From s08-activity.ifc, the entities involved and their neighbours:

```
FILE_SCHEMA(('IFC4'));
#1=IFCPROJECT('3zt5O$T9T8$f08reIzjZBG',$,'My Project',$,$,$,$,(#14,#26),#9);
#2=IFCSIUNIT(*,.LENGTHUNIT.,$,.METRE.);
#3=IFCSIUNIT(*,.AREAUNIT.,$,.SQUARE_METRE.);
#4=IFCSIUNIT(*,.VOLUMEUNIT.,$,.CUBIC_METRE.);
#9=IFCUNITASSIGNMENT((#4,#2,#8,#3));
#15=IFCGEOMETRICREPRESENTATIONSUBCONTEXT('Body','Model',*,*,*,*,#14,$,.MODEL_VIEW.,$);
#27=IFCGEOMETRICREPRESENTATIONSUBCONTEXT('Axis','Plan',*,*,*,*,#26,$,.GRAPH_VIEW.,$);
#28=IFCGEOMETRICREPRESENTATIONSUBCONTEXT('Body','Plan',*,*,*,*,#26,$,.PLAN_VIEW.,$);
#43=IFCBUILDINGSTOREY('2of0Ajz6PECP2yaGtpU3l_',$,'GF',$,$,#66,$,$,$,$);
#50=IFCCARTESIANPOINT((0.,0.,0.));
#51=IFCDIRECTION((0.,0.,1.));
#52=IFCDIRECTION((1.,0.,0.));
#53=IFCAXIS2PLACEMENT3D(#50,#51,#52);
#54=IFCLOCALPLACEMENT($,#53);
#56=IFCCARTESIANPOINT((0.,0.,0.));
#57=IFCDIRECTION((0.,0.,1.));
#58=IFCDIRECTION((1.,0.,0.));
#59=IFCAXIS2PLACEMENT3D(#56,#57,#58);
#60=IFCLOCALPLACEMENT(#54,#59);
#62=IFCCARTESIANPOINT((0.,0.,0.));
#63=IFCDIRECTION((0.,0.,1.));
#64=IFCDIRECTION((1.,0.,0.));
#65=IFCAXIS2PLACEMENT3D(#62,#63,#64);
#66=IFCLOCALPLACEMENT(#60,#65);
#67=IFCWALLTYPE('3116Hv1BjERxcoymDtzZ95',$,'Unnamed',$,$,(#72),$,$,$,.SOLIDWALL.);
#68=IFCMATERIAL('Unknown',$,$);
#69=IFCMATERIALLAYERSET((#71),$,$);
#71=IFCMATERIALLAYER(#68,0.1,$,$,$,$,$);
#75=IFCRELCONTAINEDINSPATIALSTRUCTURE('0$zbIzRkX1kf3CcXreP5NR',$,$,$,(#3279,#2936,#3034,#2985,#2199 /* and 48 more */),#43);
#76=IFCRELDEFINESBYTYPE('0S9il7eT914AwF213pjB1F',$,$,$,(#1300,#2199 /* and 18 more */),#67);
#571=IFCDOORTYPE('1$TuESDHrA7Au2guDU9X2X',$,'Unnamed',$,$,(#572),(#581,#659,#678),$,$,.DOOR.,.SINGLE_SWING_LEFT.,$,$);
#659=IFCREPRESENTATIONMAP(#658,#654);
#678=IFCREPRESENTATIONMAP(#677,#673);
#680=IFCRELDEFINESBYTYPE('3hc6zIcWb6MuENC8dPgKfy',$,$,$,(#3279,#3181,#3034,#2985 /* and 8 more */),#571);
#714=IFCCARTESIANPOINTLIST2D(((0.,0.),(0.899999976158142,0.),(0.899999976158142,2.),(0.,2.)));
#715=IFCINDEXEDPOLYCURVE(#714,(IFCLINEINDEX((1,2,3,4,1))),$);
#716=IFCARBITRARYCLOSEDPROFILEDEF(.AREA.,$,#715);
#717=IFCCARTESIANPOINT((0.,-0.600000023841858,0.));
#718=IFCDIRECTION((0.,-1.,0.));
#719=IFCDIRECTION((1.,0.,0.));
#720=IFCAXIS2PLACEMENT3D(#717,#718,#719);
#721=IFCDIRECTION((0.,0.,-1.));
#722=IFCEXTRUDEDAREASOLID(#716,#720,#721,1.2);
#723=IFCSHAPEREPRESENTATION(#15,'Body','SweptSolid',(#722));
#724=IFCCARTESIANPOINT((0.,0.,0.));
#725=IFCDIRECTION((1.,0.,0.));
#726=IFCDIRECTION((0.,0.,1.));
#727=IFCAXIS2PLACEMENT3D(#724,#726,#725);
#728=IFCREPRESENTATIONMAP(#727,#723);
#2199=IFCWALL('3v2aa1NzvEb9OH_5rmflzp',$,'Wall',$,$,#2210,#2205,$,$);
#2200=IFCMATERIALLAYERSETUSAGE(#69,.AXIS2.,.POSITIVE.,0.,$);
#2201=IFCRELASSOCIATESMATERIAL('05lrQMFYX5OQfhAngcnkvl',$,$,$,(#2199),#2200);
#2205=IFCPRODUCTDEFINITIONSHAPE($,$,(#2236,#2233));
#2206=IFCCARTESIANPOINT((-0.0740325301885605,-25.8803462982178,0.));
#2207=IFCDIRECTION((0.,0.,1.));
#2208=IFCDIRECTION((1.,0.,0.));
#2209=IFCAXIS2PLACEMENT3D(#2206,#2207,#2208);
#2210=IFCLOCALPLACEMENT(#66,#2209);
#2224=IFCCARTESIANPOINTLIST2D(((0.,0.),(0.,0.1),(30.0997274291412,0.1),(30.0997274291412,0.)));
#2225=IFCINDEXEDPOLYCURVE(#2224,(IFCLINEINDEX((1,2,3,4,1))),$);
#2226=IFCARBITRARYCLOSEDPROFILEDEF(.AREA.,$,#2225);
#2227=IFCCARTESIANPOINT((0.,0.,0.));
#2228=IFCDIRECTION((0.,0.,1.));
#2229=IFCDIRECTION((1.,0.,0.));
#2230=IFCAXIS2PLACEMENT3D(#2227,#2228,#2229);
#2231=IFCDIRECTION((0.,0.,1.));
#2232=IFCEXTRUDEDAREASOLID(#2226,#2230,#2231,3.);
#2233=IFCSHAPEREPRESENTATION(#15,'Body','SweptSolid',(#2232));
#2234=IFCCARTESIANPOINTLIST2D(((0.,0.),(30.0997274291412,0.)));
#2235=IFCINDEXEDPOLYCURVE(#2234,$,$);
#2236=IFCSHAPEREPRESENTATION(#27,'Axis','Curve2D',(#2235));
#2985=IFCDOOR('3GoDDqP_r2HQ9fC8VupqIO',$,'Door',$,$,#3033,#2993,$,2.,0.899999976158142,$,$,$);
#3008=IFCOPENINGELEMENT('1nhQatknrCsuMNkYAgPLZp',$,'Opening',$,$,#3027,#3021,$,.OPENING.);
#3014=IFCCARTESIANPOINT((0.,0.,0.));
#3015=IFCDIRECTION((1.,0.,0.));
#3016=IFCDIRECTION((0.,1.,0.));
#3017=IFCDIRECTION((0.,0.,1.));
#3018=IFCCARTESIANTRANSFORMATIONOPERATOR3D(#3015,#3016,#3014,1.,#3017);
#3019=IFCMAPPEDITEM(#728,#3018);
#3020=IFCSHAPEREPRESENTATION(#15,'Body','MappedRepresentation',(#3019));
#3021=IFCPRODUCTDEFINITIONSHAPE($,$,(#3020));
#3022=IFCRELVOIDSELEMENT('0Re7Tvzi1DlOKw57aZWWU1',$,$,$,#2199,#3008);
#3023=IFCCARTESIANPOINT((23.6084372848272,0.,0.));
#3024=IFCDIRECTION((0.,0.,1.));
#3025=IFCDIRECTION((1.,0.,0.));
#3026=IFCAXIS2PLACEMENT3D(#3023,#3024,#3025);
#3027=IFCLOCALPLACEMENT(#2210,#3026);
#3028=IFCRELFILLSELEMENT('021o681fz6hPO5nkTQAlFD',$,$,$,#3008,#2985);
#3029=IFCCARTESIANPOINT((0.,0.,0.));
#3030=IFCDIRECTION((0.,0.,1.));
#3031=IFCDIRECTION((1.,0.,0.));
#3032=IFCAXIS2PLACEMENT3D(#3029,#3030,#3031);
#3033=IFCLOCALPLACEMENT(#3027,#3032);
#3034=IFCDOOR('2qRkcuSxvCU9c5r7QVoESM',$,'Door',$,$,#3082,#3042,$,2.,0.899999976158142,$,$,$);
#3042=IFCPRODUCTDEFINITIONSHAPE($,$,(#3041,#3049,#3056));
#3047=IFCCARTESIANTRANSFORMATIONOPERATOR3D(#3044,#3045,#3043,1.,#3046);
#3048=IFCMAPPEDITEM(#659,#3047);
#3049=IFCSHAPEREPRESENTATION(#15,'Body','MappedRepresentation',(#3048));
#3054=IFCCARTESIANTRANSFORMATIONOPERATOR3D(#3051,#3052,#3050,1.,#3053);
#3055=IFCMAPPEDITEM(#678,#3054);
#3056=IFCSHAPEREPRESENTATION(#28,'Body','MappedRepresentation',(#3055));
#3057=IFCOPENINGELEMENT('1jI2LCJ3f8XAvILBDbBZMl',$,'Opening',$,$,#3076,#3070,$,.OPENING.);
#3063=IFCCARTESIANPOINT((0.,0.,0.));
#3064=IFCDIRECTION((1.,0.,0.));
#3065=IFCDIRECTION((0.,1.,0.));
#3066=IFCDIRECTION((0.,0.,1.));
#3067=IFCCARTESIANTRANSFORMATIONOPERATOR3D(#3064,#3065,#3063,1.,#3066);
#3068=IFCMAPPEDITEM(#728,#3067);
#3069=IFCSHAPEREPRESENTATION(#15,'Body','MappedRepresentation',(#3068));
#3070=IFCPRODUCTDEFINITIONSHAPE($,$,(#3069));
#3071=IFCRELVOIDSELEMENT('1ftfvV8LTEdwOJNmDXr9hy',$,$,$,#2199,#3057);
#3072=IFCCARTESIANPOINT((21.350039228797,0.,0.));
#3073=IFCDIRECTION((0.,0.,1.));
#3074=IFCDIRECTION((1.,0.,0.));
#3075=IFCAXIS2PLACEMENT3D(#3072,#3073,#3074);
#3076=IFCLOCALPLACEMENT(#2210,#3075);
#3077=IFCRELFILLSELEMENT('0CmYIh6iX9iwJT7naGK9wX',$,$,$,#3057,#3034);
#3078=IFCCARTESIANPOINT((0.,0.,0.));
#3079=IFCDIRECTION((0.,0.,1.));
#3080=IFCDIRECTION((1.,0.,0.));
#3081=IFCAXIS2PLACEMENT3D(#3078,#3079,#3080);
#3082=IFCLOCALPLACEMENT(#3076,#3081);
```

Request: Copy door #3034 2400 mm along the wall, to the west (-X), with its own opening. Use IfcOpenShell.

```python
import ifcopenshell
import ifcopenshell.api.feature
import ifcopenshell.api.geometry
import ifcopenshell.api.root
import ifcopenshell.geom
import ifcopenshell.util.element
import ifcopenshell.util.placement
import ifcopenshell.util.shape
import ifcopenshell.util.unit

model = ifcopenshell.open("s08-activity.ifc")
unit_scale = ifcopenshell.util.unit.calculate_unit_scale(model)
settings = ifcopenshell.geom.settings()


def volume(element):
    """Net volume in cubic metres, openings subtracted."""
    shape = ifcopenshell.geom.create_shape(settings, element)
    return ifcopenshell.util.shape.get_volume(shape.geometry)


door = model.by_id(3034)
opening = door.FillsVoids[0].RelatingOpeningElement
wall = opening.VoidsElements[0].RelatingBuildingElement
before = volume(wall)
shift = ifcopenshell.util.placement.get_local_placement(wall.ObjectPlacement)[:3, 0] * -2.4 / unit_scale

# copy_class copies the void relationship, type, container and properties, but no geometry.
new_opening = ifcopenshell.api.root.copy_class(model, product=opening)
new_opening.Representation = ifcopenshell.util.element.copy_deep(
    model, opening.Representation, exclude=["IfcGeometricRepresentationContext", "IfcRepresentationMap"]
)
new_door = ifcopenshell.api.root.copy_class(model, product=door)
new_door.Representation = ifcopenshell.util.element.copy_deep(
    model, door.Representation, exclude=["IfcGeometricRepresentationContext", "IfcRepresentationMap"]
)
ifcopenshell.api.feature.add_filling(model, opening=new_opening, element=new_door)

for old, new in ((opening, new_opening), (door, new_door)):
    matrix = ifcopenshell.util.placement.get_local_placement(old.ObjectPlacement)
    matrix[:3, 3] += shift
    ifcopenshell.api.geometry.edit_object_placement(model, product=new, matrix=matrix, is_si=False)

after = volume(wall)

print(f"wall volume {before:.3f} -> {after:.3f} m3")

model.write("s08-activity-out.ifc")
```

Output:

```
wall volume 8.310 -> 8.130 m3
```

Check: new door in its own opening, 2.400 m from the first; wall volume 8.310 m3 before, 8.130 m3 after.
